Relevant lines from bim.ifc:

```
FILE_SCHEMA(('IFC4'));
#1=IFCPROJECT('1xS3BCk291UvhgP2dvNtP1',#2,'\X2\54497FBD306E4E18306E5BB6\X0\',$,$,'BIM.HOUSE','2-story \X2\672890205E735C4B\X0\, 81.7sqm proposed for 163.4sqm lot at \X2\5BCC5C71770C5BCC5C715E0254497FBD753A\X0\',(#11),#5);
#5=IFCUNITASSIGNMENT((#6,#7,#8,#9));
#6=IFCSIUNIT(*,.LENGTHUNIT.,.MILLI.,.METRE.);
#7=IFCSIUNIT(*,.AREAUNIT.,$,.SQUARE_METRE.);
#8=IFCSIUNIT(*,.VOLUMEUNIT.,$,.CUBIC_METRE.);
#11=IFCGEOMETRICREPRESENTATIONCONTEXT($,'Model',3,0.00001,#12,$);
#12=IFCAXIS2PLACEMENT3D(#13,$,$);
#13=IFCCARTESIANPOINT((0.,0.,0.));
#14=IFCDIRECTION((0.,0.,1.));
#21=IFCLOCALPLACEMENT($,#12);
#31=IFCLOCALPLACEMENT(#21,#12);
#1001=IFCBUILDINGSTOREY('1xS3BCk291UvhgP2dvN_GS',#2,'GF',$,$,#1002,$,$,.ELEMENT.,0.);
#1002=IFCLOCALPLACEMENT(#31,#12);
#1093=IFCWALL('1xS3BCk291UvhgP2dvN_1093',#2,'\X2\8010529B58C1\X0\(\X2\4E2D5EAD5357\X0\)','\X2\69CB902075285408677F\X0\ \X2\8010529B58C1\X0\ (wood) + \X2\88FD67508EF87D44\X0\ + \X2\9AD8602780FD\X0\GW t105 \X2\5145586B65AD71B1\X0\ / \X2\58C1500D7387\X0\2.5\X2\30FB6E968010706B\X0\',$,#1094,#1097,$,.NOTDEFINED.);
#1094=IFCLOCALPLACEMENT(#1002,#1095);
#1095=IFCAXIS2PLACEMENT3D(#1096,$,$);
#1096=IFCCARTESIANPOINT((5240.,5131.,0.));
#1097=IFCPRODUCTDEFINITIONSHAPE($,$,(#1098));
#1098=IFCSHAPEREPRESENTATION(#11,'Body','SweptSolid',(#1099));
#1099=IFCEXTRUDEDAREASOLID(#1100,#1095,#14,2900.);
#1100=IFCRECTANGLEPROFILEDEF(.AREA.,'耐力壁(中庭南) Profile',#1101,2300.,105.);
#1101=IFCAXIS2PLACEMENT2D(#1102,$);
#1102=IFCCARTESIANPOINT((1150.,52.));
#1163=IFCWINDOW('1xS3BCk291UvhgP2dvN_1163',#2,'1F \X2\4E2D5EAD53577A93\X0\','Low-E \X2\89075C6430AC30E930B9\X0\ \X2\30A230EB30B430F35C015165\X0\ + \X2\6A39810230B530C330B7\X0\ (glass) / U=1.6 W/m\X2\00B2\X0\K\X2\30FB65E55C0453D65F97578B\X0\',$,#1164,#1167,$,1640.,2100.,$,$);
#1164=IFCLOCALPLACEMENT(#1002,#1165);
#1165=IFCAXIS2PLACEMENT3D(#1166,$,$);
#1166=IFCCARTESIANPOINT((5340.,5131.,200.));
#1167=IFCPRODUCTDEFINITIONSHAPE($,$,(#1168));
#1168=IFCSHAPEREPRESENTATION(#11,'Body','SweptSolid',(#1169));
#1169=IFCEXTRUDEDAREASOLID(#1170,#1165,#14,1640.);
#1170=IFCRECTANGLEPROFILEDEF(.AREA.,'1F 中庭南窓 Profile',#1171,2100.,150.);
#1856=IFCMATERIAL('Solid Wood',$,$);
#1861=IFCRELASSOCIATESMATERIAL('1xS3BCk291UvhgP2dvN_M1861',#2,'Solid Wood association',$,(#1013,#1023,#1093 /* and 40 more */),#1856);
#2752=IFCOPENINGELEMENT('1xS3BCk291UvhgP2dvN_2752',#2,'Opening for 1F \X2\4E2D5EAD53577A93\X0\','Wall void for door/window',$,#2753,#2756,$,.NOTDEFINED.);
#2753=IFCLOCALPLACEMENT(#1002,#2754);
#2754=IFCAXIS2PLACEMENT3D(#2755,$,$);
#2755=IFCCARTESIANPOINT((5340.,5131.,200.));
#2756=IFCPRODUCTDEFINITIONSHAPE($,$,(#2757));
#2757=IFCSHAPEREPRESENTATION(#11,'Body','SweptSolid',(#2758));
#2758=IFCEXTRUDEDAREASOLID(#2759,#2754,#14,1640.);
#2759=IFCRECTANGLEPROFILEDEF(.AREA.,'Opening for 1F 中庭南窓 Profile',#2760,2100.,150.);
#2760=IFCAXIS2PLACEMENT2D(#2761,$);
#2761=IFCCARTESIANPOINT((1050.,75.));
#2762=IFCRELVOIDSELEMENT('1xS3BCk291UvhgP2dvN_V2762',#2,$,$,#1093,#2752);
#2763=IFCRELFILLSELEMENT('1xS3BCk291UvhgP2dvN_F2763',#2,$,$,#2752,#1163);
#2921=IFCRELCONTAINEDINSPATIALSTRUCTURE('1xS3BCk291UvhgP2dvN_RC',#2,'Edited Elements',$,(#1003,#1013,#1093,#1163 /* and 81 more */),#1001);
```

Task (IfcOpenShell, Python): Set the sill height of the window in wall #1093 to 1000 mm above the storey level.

```python
import numpy as np
import ifcopenshell
import ifcopenshell.api.geometry
import ifcopenshell.geom
import ifcopenshell.util.element
import ifcopenshell.util.placement
import ifcopenshell.util.shape
import ifcopenshell.util.unit

model = ifcopenshell.open("bim.ifc")
unit_scale = ifcopenshell.util.unit.calculate_unit_scale(model)

window = model.by_guid("1xS3BCk291UvhgP2dvN_1163")
opening = window.FillsVoids[0].RelatingOpeningElement
storey = ifcopenshell.util.element.get_container(window, ifc_class="IfcBuildingStorey")
level = ifcopenshell.util.placement.get_local_placement(storey.ObjectPlacement)[2, 3]

# The opening's origin need not be at the sill, so measure its lowest point.
shape = ifcopenshell.geom.create_shape(ifcopenshell.geom.settings(), opening)
bottom = ifcopenshell.util.shape.get_shape_bottom_elevation(shape, shape.geometry) / unit_scale
dz = level + 1 / unit_scale - bottom

shift = np.array([0.0, 0.0, dz])
# The window is not placed relative to its opening, so move both.
for product in (opening, window):
    matrix = ifcopenshell.util.placement.get_local_placement(product.ObjectPlacement)
    matrix[:3, 3] += shift
    ifcopenshell.api.geometry.edit_object_placement(model, product=product, matrix=matrix, is_si=False)

print(f"moved by {dz * unit_scale:+.3f} m")

model.write("bim-out.ifc")
```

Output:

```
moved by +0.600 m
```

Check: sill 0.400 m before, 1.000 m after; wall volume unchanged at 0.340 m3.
